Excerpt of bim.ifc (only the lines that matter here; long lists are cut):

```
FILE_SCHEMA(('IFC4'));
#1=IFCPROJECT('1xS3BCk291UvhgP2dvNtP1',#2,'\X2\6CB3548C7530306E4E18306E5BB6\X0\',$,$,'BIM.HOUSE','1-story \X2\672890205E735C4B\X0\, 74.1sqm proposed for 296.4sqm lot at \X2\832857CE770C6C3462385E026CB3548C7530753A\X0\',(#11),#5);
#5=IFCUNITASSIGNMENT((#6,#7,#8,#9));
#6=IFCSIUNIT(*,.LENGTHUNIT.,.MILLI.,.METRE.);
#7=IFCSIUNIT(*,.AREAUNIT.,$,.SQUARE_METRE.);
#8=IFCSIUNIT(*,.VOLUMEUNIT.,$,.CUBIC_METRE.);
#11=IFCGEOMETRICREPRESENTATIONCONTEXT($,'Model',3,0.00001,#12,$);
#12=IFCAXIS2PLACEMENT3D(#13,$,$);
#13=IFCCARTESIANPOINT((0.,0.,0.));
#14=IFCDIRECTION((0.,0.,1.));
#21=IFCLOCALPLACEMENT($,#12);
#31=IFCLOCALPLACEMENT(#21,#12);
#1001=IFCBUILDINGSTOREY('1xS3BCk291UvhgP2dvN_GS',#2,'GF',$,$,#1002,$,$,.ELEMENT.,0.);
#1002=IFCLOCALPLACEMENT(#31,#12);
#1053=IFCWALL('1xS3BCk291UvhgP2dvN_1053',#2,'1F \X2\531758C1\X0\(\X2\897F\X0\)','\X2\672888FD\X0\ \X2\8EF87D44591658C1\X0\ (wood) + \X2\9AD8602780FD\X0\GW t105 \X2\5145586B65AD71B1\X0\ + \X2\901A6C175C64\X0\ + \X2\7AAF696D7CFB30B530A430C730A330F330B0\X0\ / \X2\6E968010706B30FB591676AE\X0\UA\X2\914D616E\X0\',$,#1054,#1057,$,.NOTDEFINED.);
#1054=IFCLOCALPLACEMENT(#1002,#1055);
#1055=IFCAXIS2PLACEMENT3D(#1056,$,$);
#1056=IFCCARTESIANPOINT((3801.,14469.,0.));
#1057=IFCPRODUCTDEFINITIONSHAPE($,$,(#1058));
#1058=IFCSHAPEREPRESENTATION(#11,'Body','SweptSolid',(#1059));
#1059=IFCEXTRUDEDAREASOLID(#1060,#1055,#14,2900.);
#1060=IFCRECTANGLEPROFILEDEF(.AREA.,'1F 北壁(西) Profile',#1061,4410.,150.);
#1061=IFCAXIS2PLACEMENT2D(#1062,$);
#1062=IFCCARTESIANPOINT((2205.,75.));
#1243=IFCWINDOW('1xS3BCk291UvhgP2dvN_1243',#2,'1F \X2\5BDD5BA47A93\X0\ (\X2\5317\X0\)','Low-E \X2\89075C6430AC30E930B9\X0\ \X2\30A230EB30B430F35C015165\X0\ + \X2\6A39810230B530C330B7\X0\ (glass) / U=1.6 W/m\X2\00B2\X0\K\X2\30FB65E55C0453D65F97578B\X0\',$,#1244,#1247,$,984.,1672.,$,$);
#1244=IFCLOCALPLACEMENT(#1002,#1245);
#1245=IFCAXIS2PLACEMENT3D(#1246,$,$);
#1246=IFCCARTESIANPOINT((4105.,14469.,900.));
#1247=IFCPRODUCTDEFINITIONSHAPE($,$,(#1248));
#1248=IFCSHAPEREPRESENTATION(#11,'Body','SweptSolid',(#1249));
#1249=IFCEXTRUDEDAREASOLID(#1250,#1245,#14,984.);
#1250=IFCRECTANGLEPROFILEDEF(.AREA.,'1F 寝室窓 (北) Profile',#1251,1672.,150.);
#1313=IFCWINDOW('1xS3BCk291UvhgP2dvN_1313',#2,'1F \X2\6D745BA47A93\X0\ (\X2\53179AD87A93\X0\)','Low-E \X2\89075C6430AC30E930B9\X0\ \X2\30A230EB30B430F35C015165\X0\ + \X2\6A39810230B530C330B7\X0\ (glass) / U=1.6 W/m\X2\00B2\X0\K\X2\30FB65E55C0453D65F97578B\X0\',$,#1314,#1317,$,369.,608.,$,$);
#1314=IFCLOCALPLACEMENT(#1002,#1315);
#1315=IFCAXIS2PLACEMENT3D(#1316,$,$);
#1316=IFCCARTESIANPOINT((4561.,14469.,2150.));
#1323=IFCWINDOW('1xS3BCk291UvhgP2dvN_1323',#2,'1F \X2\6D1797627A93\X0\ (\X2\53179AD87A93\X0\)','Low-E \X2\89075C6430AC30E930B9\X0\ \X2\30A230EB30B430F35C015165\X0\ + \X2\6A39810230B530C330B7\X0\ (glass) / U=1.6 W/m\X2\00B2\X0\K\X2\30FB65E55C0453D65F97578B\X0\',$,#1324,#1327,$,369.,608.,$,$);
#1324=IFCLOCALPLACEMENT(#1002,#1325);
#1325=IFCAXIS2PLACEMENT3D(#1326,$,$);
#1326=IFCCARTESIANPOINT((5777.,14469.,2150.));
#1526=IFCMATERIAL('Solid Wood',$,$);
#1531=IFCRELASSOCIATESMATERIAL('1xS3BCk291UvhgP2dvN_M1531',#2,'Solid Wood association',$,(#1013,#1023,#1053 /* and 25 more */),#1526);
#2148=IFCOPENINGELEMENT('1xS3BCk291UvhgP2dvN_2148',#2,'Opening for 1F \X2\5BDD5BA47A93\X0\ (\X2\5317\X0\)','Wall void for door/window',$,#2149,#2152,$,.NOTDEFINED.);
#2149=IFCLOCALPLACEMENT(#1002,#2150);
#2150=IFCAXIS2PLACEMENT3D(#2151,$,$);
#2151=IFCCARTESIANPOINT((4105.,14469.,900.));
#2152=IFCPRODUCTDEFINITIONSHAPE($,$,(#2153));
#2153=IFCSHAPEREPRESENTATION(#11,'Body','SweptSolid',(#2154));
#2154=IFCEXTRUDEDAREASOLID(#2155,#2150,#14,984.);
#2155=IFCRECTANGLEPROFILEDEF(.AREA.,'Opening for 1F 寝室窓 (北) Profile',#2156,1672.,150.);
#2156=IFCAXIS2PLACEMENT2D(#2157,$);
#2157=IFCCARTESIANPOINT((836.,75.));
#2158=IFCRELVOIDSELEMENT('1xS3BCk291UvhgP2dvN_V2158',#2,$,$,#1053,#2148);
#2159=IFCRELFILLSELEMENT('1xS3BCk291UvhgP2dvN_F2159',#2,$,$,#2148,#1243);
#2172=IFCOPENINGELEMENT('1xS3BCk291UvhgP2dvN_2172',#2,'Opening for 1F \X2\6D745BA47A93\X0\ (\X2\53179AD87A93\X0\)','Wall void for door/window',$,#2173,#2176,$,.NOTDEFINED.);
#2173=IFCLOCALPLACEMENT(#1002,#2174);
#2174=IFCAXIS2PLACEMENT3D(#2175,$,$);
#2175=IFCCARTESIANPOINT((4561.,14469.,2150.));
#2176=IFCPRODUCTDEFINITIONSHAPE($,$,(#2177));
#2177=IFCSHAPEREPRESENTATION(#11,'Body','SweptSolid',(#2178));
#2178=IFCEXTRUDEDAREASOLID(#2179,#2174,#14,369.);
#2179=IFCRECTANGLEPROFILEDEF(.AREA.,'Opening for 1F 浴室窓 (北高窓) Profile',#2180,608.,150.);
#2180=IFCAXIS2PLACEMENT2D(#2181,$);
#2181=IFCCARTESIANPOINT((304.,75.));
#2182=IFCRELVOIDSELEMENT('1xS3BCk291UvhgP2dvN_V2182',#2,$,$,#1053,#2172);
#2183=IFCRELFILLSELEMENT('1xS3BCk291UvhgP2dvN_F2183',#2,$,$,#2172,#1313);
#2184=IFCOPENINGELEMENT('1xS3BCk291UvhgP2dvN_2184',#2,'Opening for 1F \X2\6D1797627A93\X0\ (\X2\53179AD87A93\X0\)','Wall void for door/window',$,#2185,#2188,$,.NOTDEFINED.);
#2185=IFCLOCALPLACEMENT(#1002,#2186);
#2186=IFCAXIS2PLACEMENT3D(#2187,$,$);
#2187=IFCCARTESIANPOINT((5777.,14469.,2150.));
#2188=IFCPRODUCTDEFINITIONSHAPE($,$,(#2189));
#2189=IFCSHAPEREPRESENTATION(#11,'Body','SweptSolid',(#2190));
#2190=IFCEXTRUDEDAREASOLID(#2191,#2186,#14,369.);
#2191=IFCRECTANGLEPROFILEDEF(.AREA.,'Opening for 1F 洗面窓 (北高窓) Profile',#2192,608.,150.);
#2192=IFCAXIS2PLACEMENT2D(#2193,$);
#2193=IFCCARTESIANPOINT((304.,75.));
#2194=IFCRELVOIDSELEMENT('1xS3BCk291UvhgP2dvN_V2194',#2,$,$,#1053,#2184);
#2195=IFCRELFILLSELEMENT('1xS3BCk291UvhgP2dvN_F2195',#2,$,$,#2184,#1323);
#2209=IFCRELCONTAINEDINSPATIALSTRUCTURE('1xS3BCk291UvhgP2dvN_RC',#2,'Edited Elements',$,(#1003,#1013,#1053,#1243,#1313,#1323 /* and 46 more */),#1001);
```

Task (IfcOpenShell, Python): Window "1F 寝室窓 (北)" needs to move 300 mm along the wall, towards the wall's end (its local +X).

```python
import ifcopenshell
import ifcopenshell.api.geometry
import ifcopenshell.util.placement
import ifcopenshell.util.unit

model = ifcopenshell.open("bim.ifc")
unit_scale = ifcopenshell.util.unit.calculate_unit_scale(model)

window = model.by_guid("1xS3BCk291UvhgP2dvN_1243")
opening = window.FillsVoids[0].RelatingOpeningElement
wall = opening.VoidsElements[0].RelatingBuildingElement

wall_matrix = ifcopenshell.util.placement.get_local_placement(wall.ObjectPlacement)
shift = wall_matrix[:3, 0] * 0.3 / unit_scale
before = ifcopenshell.util.placement.get_local_placement(window.ObjectPlacement)[:3, 3].copy()

# The window is not placed relative to its opening, so move both.
for product in (opening, window):
    matrix = ifcopenshell.util.placement.get_local_placement(product.ObjectPlacement)
    matrix[:3, 3] += shift
    ifcopenshell.api.geometry.edit_object_placement(model, product=product, matrix=matrix, is_si=False)

after = ifcopenshell.util.placement.get_local_placement(window.ObjectPlacement)[:3, 3]
print("window moved by", (after - before).round(3) + 0.0)

model.write("bim_rev.ifc")
```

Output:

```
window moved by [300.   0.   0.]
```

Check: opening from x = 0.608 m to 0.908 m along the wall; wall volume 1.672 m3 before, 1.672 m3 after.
